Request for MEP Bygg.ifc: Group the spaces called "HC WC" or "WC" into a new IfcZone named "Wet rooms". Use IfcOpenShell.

First a look at what the model holds.

```python
import ifcopenshell

model = ifcopenshell.open("MEP Bygg.ifc")
print(model.schema)
seen = {}
for space in model.by_type("IfcSpace"):
    seen[space.LongName] = seen.get(space.LongName, 0) + 1
for name, count in sorted(seen.items(), key=str):
    print(count, "x", name)
print("zones:", [z.Name for z in model.by_type("IfcZone")][:20])
```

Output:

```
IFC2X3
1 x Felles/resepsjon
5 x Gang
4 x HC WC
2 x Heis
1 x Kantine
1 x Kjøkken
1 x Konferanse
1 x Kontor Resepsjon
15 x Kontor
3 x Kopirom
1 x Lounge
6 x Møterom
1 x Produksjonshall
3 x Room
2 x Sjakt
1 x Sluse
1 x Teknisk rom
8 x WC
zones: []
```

```python
import ifcopenshell
import ifcopenshell.api.group
import ifcopenshell.api.root

model = ifcopenshell.open("MEP Bygg.ifc")

names = {"HC WC", "WC"}
spaces = [s for s in model.by_type("IfcSpace") if s.LongName in names]

zone = ifcopenshell.api.root.create_entity(model, ifc_class="IfcZone", name="Wet rooms")
ifcopenshell.api.group.assign_group(model, products=spaces, group=zone)
print(len(spaces), "spaces in", zone.Name)

model.write("MEP Bygg_edited.ifc")
```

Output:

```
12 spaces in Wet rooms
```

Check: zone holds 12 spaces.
